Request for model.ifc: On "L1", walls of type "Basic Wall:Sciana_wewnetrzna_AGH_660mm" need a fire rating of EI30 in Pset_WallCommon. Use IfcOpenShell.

First a look at what the model holds.

```python
import ifcopenshell
import ifcopenshell.util.element

model = ifcopenshell.open("model.ifc")
print(model.schema)
storey = next(s for s in model.by_type("IfcBuildingStorey") if s.Name == "L1")
walls = [e for e in ifcopenshell.util.element.get_decomposition(storey) if e.is_a("IfcWall")]
seen = {}
for e in walls:
    element_type = ifcopenshell.util.element.get_type(e)
    key = (element_type.Name if element_type != e and element_type else None, ifcopenshell.util.element.get_pset(e, "Pset_WallCommon", "FireRating"))
    seen[key] = seen.get(key, 0) + 1
for (name, value), count in sorted(seen.items(), key=str):
    print(count, "x", name, "|", value)
```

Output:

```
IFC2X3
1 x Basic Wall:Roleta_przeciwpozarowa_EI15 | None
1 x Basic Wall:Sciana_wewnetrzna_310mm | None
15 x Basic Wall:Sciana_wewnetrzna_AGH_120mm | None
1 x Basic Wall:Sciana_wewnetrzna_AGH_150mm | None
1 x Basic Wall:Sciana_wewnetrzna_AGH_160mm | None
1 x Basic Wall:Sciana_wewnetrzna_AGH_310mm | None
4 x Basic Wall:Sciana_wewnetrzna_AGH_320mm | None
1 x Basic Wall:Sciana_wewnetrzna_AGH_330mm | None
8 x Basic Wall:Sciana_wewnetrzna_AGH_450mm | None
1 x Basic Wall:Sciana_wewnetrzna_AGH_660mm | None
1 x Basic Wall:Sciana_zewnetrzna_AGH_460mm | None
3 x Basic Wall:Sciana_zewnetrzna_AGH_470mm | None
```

```python
import ifcopenshell
import ifcopenshell.api.pset
import ifcopenshell.util.element

model = ifcopenshell.open("model.ifc")

storey = next(s for s in model.by_type("IfcBuildingStorey") if s.Name == "L1")
walls = [e for e in ifcopenshell.util.element.get_decomposition(storey) if e.is_a("IfcWall")]

count = 0
for e in walls:
    element_type = ifcopenshell.util.element.get_type(e)
    if element_type in (None, e) or element_type.Name != "Basic Wall:Sciana_wewnetrzna_AGH_660mm":
        continue
    # add_pset returns the element's existing set when there is one.
    pset = ifcopenshell.api.pset.add_pset(model, product=e, name="Pset_WallCommon")
    ifcopenshell.api.pset.edit_pset(model, pset=pset, properties={"FireRating": "EI30"})
    count += 1

print(count, "walls updated")

model.write("model-out.ifc")
```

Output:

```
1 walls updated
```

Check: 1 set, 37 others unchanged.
